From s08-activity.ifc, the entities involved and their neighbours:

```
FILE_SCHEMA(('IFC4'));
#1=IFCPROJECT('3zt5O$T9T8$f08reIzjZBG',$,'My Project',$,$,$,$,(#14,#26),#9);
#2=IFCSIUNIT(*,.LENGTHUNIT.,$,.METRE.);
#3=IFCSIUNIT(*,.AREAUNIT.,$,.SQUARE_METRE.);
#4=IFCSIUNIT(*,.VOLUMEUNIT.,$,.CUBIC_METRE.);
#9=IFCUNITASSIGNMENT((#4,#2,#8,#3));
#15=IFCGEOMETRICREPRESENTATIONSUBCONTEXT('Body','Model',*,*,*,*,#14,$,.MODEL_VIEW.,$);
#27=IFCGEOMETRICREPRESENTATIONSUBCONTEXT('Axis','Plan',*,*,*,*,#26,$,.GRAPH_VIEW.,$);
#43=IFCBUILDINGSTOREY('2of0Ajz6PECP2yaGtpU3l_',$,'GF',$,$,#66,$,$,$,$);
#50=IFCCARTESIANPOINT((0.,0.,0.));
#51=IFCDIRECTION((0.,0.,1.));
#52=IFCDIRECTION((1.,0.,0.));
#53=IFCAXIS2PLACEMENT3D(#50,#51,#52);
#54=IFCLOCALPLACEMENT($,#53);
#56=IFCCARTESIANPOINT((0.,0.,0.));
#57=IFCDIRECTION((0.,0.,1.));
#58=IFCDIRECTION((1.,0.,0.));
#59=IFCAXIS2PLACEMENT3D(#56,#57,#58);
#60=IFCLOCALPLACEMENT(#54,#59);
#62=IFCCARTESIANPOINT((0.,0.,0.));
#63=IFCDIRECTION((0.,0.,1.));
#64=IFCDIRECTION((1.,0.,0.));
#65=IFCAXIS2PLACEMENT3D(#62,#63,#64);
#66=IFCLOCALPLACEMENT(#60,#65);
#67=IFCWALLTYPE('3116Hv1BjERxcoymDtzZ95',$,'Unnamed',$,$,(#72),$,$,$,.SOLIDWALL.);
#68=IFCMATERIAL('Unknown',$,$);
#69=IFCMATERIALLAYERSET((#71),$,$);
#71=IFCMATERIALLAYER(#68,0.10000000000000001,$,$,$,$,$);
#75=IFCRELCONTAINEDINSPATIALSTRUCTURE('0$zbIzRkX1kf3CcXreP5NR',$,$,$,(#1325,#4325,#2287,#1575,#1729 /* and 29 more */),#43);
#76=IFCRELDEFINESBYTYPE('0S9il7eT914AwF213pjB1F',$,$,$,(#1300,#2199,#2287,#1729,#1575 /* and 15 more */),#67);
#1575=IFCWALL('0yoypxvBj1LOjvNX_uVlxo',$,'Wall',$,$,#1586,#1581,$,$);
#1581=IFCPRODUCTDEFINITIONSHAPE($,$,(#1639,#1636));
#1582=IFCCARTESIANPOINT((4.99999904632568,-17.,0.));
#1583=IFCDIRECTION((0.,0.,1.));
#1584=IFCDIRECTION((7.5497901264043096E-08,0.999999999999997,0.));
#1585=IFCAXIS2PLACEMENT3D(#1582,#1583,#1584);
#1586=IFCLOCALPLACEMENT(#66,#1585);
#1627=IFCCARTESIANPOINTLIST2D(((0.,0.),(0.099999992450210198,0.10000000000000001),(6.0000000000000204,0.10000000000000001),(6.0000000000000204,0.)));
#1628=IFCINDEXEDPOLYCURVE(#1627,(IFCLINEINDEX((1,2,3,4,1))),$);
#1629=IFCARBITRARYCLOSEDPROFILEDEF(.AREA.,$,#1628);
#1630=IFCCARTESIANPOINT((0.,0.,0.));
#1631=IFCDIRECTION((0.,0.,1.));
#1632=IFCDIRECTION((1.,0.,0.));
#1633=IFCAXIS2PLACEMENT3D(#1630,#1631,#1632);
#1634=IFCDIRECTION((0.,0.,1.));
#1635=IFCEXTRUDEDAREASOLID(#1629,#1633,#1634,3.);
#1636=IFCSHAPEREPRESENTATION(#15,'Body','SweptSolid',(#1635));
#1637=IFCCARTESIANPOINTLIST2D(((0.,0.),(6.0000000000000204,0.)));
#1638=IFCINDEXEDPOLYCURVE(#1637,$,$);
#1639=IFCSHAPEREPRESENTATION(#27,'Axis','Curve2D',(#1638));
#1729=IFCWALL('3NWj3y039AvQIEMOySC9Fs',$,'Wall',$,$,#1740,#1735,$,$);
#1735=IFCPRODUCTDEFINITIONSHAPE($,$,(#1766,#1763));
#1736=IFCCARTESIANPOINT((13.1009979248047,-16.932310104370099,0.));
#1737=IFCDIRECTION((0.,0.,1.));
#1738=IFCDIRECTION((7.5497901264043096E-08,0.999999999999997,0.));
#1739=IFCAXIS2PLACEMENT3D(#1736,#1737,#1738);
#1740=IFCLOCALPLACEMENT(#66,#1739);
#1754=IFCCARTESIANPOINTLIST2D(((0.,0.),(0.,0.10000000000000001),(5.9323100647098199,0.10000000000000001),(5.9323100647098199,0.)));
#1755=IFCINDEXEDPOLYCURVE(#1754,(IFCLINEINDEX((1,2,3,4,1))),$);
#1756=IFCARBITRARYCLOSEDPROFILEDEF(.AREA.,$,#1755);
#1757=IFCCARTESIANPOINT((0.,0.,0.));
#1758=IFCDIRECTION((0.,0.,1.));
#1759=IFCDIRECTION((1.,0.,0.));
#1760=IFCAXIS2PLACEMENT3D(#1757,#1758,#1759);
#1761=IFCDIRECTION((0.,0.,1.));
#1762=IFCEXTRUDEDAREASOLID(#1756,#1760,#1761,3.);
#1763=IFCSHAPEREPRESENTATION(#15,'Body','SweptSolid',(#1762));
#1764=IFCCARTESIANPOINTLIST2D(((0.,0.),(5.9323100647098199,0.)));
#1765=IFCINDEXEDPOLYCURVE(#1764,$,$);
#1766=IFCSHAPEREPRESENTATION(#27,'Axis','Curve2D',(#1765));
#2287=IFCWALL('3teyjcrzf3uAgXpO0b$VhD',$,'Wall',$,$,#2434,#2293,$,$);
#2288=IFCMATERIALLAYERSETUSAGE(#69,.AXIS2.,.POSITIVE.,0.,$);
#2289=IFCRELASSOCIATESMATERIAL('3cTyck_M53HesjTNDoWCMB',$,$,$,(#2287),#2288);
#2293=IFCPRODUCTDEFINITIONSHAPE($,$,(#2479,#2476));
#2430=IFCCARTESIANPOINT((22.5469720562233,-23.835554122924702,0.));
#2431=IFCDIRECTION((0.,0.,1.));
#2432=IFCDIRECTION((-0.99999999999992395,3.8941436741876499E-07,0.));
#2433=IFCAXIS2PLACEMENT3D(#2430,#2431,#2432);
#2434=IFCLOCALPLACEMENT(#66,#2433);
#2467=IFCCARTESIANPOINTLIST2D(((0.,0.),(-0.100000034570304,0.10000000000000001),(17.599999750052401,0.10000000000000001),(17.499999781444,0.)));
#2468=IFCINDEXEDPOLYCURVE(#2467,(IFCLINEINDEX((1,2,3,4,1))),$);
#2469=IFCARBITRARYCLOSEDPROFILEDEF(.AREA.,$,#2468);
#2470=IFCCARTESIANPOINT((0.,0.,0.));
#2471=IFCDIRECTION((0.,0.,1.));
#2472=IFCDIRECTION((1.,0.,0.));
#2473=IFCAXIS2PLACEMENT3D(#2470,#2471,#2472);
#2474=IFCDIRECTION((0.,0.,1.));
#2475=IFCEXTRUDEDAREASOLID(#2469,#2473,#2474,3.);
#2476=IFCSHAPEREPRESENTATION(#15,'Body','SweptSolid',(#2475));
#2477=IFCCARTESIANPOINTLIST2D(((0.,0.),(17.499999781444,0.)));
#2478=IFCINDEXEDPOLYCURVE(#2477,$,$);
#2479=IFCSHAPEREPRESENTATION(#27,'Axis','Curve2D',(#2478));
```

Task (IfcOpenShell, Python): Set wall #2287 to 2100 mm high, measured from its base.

```python
import ifcopenshell
import ifcopenshell.geom
import ifcopenshell.util.representation
import ifcopenshell.util.shape

model = ifcopenshell.open("s08-activity.ifc")
settings = ifcopenshell.geom.settings()


def volume(element):
    """Net volume in cubic metres, openings subtracted."""
    shape = ifcopenshell.geom.create_shape(settings, element)
    return ifcopenshell.util.shape.get_volume(shape.geometry)


wall = model.by_guid("3teyjcrzf3uAgXpO0b$VhD")
before = volume(wall)

body = ifcopenshell.util.representation.get_representation(wall, "Model", "Body")
solid = body.Items[0]
old_height = solid.Depth
solid.Depth = 2.1
after = volume(wall)

print(f"height {old_height:g} -> {solid.Depth:g}, volume {before:.3f} -> {after:.3f} m3")

model.write("s08-activity_edited.ifc")
```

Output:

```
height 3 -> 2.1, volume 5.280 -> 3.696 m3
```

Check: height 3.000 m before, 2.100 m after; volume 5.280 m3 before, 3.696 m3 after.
